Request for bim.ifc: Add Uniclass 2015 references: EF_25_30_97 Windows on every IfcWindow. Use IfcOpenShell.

First a look at what the model holds.

```python
import ifcopenshell

model = ifcopenshell.open("bim.ifc")
print(model.schema)
print("classifications:", [c.Name for c in model.by_type("IfcClassification")])
for ifc_class in ("IfcDoor", "IfcRoof", "IfcStair", "IfcWall", "IfcWindow"):
    print(ifc_class, len(model.by_type(ifc_class)))
```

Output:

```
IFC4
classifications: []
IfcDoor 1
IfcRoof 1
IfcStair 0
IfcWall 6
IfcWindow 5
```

```python
import ifcopenshell
import ifcopenshell.api.classification

model = ifcopenshell.open("bim.ifc")

system = ifcopenshell.api.classification.add_classification(model, classification="Uniclass 2015")

codes = {
    "IfcWindow": ("EF_25_30_97", "Windows"),
}
for ifc_class, (code, name) in codes.items():
    products = model.by_type(ifc_class)
    ifcopenshell.api.classification.add_reference(
        model, products=products, classification=system, identification=code, name=name
    )
    print(code, len(products))

model.write("bim-out.ifc")
```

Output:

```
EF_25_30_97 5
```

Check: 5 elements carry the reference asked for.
